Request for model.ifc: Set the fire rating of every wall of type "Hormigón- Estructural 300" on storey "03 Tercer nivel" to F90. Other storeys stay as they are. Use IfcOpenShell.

First a look at what the model holds.

```python
import ifcopenshell
import ifcopenshell.util.element

model = ifcopenshell.open("model.ifc")
print(model.schema)
storey = next(s for s in model.by_type("IfcBuildingStorey") if s.Name == "03 Tercer nivel")
walls = [e for e in ifcopenshell.util.element.get_decomposition(storey) if e.is_a("IfcWall")]
seen = {}
for e in walls:
    element_type = ifcopenshell.util.element.get_type(e)
    key = (element_type.Name if element_type != e and element_type else None, ifcopenshell.util.element.get_pset(e, "Pset_WallCommon", "FireRating"))
    seen[key] = seen.get(key, 0) + 1
for (name, value), count in sorted(seen.items(), key=str):
    print(count, "x", name, "|", value)
```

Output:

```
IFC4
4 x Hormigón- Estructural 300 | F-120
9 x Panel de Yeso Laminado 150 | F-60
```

```python
import ifcopenshell
import ifcopenshell.api.pset
import ifcopenshell.util.element

model = ifcopenshell.open("model.ifc")

storey = next(s for s in model.by_type("IfcBuildingStorey") if s.Name == "03 Tercer nivel")
walls = [e for e in ifcopenshell.util.element.get_decomposition(storey) if e.is_a("IfcWall")]

count = 0
for e in walls:
    element_type = ifcopenshell.util.element.get_type(e)
    if element_type in (None, e) or element_type.Name != "Hormigón- Estructural 300":
        continue
    # add_pset returns the element's existing set when there is one.
    pset = ifcopenshell.api.pset.add_pset(model, product=e, name="Pset_WallCommon")
    ifcopenshell.api.pset.edit_pset(model, pset=pset, properties={"FireRating": "F90"})
    count += 1

print(count, "walls updated")

model.write("model_rev.ifc")
```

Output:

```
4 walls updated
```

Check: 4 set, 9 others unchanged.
